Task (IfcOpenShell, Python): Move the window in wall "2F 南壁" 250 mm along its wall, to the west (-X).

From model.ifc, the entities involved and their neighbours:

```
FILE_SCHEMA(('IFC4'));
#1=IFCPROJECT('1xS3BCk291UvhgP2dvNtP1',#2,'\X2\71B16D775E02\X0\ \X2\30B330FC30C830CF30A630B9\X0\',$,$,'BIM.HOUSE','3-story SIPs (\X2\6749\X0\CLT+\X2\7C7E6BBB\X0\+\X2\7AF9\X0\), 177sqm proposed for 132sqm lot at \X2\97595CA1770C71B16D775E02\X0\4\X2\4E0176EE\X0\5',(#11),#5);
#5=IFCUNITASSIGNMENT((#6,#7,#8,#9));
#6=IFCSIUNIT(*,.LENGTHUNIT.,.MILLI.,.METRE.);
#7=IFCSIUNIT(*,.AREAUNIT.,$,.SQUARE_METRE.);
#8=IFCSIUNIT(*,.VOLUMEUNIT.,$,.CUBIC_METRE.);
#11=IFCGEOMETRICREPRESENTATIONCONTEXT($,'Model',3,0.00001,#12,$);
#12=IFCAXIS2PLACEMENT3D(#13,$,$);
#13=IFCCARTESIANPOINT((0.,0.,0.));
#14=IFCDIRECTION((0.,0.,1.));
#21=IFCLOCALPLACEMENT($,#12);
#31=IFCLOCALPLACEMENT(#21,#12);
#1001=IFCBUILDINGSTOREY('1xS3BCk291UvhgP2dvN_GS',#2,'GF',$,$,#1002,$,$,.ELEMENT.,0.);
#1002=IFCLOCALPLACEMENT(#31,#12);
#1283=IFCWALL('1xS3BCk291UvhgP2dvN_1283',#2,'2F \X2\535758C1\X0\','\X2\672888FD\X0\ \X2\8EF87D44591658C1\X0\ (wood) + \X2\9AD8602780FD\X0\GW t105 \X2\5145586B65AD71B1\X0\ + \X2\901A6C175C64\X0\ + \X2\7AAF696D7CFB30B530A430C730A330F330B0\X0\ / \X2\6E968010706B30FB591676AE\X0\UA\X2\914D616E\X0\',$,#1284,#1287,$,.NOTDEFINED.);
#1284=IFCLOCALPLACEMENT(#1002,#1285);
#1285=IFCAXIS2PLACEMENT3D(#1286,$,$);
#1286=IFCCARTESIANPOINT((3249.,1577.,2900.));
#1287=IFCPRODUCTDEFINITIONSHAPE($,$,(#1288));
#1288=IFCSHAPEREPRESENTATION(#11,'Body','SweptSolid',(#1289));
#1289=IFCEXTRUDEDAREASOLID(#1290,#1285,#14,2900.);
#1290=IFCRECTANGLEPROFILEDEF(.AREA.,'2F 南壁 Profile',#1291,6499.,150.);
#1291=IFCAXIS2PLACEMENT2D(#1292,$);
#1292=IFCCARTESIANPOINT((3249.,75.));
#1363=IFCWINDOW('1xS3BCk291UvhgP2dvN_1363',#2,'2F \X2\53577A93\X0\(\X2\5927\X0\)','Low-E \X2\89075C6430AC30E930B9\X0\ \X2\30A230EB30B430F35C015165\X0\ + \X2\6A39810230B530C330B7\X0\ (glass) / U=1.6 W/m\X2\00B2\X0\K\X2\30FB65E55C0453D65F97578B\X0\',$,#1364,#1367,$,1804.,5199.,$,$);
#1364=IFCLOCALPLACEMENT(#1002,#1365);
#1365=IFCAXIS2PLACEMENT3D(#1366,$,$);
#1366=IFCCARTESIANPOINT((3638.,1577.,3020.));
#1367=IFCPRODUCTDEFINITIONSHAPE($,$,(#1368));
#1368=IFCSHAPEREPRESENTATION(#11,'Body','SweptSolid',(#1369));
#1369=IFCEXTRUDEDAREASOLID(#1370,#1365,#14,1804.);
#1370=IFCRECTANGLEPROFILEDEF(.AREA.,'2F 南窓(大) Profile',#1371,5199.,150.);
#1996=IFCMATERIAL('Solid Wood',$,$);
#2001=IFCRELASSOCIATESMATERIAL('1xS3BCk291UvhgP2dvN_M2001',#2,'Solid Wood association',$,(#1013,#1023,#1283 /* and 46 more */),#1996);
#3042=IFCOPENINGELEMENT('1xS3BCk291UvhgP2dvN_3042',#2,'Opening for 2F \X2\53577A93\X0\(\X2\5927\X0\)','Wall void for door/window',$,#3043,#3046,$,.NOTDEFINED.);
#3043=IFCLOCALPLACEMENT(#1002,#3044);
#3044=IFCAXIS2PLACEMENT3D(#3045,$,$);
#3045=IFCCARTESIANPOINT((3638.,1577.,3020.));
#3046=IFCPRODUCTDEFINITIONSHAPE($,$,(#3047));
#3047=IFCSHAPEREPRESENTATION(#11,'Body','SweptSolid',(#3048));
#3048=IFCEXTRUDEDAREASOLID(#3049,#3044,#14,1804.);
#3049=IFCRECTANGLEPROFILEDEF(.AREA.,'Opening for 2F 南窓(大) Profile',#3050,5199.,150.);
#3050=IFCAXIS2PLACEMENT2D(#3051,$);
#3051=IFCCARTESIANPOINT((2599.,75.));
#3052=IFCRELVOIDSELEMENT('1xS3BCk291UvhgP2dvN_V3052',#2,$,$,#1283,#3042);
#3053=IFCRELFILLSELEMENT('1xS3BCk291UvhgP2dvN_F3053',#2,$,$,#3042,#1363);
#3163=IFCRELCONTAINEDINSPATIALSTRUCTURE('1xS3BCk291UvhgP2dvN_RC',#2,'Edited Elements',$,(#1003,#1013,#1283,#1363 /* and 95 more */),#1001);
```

```python
import ifcopenshell
import ifcopenshell.api.geometry
import ifcopenshell.util.placement
import ifcopenshell.util.unit

model = ifcopenshell.open("model.ifc")
unit_scale = ifcopenshell.util.unit.calculate_unit_scale(model)

window = model.by_guid("1xS3BCk291UvhgP2dvN_1363")
opening = window.FillsVoids[0].RelatingOpeningElement
wall = opening.VoidsElements[0].RelatingBuildingElement

wall_matrix = ifcopenshell.util.placement.get_local_placement(wall.ObjectPlacement)
shift = wall_matrix[:3, 0] * -0.25 / unit_scale
before = ifcopenshell.util.placement.get_local_placement(window.ObjectPlacement)[:3, 3].copy()

# The window is not placed relative to its opening, so move both.
for product in (opening, window):
    matrix = ifcopenshell.util.placement.get_local_placement(product.ObjectPlacement)
    matrix[:3, 3] += shift
    ifcopenshell.api.geometry.edit_object_placement(model, product=product, matrix=matrix, is_si=False)

after = ifcopenshell.util.placement.get_local_placement(window.ObjectPlacement)[:3, 3]
print("window moved by", (after - before).round(3) + 0.0)

model.write("model_edited.ifc")
```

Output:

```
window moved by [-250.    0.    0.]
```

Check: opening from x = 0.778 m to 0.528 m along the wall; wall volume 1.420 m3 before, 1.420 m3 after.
